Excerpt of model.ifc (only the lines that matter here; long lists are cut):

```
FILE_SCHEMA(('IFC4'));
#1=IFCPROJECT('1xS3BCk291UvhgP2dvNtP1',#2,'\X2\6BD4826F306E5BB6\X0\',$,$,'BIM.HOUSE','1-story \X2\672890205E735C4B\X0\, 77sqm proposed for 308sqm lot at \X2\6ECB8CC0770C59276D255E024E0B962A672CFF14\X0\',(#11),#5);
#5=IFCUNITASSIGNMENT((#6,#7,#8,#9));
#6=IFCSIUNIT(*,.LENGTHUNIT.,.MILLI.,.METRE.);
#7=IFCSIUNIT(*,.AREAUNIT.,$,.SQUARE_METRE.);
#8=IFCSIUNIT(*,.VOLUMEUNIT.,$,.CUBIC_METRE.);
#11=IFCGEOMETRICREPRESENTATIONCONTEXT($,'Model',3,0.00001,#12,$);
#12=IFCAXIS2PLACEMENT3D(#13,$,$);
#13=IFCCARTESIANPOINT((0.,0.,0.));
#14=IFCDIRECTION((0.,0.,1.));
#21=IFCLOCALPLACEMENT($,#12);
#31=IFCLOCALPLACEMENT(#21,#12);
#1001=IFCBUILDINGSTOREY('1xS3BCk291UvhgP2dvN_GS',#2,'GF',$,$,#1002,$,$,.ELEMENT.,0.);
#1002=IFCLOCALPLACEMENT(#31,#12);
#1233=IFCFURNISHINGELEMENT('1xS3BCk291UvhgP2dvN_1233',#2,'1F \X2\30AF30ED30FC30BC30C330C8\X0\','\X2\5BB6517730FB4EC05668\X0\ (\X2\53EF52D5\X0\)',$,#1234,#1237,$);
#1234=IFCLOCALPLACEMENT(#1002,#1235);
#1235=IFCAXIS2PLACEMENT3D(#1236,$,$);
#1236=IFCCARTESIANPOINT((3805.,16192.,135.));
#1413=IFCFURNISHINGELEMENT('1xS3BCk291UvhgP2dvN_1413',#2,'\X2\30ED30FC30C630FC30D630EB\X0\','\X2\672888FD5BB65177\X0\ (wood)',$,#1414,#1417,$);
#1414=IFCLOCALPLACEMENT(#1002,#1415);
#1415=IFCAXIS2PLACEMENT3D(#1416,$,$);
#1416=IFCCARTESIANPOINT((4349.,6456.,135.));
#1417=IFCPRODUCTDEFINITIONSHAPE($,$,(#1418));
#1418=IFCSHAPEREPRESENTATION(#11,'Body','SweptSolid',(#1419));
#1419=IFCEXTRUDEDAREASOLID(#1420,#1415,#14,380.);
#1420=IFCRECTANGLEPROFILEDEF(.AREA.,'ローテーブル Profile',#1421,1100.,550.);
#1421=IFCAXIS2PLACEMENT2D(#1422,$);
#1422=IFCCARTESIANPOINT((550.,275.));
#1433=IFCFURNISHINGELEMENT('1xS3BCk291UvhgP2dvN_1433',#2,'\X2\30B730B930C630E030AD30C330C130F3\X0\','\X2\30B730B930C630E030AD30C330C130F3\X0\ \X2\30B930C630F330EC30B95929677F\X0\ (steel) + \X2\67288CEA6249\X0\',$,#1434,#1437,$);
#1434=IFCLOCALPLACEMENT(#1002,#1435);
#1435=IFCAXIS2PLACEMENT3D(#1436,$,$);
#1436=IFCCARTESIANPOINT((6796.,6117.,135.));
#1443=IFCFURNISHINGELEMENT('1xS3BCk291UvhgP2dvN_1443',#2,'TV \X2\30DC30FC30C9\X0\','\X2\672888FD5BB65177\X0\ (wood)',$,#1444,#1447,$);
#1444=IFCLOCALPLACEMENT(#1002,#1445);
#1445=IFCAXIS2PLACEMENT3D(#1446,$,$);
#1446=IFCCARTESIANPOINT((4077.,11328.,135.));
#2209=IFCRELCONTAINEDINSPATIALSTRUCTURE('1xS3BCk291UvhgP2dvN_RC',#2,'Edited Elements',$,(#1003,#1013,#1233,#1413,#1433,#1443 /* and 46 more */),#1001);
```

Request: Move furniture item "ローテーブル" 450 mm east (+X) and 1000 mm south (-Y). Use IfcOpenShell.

```python
import ifcopenshell
import ifcopenshell.api.geometry
import ifcopenshell.util.placement
import ifcopenshell.util.unit

model = ifcopenshell.open("model.ifc")
unit_scale = ifcopenshell.util.unit.calculate_unit_scale(model)

item = model.by_guid("1xS3BCk291UvhgP2dvN_1413")
matrix = ifcopenshell.util.placement.get_local_placement(item.ObjectPlacement)
matrix[0, 3] += 0.45 / unit_scale
matrix[1, 3] -= 1 / unit_scale
ifcopenshell.api.geometry.edit_object_placement(model, product=item, matrix=matrix, is_si=False)

print(ifcopenshell.util.placement.get_local_placement(item.ObjectPlacement).round(3) + 0.0)

model.write("model_updated.ifc")
```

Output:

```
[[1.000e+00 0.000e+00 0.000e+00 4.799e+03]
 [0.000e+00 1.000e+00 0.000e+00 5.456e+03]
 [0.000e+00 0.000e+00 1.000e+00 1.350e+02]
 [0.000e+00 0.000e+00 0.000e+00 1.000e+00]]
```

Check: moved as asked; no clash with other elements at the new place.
